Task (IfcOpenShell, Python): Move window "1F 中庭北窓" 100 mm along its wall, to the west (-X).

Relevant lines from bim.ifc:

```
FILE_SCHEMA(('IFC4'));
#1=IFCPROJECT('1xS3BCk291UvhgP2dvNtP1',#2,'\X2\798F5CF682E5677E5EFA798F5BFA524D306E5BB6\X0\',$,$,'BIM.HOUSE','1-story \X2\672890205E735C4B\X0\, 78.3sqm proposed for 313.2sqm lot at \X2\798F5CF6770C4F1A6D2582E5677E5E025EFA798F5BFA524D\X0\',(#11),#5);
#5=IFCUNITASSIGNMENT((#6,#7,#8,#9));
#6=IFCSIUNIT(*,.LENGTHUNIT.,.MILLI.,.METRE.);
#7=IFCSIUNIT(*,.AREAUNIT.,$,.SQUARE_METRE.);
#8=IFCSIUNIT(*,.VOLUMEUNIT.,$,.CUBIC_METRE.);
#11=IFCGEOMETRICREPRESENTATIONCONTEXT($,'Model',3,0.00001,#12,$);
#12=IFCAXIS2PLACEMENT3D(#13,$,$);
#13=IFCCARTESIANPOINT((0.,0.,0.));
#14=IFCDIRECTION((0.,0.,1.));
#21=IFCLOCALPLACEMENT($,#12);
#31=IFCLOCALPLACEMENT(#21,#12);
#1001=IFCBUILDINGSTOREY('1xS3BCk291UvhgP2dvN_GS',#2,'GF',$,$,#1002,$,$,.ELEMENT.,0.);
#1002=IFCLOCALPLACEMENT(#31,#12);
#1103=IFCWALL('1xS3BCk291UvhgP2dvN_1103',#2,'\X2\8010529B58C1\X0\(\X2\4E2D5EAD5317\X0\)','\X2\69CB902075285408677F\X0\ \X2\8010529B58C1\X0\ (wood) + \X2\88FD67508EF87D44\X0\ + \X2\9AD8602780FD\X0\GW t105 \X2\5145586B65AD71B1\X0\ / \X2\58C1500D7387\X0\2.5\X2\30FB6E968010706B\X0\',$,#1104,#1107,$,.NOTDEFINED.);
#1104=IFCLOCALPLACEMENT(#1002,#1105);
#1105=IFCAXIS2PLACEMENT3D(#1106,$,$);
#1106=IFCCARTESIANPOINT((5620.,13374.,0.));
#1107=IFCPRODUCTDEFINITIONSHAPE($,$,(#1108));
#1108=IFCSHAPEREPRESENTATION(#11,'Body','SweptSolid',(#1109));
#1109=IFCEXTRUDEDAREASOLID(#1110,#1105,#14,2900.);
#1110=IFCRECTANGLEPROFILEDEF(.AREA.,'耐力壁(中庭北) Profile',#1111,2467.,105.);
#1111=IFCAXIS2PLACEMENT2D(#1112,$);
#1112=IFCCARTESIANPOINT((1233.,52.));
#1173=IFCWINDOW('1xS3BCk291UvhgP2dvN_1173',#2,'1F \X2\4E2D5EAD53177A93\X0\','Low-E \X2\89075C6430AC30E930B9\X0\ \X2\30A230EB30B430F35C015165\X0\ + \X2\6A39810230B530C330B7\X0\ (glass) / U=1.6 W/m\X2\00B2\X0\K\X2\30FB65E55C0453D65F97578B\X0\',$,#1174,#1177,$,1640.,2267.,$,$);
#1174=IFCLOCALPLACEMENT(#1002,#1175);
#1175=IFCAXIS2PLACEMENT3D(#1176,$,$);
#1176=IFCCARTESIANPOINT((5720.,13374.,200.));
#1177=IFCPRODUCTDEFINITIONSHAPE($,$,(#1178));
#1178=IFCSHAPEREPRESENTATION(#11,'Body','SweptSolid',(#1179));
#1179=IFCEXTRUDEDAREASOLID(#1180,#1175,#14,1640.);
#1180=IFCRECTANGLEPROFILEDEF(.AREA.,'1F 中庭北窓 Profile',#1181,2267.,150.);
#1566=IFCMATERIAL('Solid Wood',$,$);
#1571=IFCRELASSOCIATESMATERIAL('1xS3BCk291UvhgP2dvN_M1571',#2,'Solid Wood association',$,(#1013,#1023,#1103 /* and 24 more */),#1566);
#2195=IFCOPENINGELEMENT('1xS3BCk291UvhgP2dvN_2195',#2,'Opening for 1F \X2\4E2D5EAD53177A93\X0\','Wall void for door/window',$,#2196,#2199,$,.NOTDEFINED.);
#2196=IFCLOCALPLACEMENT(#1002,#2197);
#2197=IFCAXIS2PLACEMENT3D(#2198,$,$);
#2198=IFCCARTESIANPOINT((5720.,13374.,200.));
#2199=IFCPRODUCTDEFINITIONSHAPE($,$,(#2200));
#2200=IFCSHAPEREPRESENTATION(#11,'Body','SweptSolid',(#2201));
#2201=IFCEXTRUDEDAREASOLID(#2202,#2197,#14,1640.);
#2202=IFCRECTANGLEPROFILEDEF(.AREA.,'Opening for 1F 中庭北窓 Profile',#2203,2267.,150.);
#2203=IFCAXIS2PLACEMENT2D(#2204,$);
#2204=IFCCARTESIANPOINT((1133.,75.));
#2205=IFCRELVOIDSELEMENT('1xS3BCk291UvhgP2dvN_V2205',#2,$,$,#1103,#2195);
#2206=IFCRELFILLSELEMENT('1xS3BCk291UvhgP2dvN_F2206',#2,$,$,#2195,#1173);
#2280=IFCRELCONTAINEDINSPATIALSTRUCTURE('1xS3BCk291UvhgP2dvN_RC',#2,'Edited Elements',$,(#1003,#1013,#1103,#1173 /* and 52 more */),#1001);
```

```python
import ifcopenshell
import ifcopenshell.api.geometry
import ifcopenshell.util.placement
import ifcopenshell.util.unit

model = ifcopenshell.open("bim.ifc")
unit_scale = ifcopenshell.util.unit.calculate_unit_scale(model)

window = model.by_guid("1xS3BCk291UvhgP2dvN_1173")
opening = window.FillsVoids[0].RelatingOpeningElement
wall = opening.VoidsElements[0].RelatingBuildingElement

wall_matrix = ifcopenshell.util.placement.get_local_placement(wall.ObjectPlacement)
shift = wall_matrix[:3, 0] * -0.1 / unit_scale
before = ifcopenshell.util.placement.get_local_placement(window.ObjectPlacement)[:3, 3].copy()

# The window is not placed relative to its opening, so move both.
for product in (opening, window):
    matrix = ifcopenshell.util.placement.get_local_placement(product.ObjectPlacement)
    matrix[:3, 3] += shift
    ifcopenshell.api.geometry.edit_object_placement(model, product=product, matrix=matrix, is_si=False)

after = ifcopenshell.util.placement.get_local_placement(window.ObjectPlacement)[:3, 3]
print("window moved by", (after - before).round(3) + 0.0)

model.write("bim_rev.ifc")
```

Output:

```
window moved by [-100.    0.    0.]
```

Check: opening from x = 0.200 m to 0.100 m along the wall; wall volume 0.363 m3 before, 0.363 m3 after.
